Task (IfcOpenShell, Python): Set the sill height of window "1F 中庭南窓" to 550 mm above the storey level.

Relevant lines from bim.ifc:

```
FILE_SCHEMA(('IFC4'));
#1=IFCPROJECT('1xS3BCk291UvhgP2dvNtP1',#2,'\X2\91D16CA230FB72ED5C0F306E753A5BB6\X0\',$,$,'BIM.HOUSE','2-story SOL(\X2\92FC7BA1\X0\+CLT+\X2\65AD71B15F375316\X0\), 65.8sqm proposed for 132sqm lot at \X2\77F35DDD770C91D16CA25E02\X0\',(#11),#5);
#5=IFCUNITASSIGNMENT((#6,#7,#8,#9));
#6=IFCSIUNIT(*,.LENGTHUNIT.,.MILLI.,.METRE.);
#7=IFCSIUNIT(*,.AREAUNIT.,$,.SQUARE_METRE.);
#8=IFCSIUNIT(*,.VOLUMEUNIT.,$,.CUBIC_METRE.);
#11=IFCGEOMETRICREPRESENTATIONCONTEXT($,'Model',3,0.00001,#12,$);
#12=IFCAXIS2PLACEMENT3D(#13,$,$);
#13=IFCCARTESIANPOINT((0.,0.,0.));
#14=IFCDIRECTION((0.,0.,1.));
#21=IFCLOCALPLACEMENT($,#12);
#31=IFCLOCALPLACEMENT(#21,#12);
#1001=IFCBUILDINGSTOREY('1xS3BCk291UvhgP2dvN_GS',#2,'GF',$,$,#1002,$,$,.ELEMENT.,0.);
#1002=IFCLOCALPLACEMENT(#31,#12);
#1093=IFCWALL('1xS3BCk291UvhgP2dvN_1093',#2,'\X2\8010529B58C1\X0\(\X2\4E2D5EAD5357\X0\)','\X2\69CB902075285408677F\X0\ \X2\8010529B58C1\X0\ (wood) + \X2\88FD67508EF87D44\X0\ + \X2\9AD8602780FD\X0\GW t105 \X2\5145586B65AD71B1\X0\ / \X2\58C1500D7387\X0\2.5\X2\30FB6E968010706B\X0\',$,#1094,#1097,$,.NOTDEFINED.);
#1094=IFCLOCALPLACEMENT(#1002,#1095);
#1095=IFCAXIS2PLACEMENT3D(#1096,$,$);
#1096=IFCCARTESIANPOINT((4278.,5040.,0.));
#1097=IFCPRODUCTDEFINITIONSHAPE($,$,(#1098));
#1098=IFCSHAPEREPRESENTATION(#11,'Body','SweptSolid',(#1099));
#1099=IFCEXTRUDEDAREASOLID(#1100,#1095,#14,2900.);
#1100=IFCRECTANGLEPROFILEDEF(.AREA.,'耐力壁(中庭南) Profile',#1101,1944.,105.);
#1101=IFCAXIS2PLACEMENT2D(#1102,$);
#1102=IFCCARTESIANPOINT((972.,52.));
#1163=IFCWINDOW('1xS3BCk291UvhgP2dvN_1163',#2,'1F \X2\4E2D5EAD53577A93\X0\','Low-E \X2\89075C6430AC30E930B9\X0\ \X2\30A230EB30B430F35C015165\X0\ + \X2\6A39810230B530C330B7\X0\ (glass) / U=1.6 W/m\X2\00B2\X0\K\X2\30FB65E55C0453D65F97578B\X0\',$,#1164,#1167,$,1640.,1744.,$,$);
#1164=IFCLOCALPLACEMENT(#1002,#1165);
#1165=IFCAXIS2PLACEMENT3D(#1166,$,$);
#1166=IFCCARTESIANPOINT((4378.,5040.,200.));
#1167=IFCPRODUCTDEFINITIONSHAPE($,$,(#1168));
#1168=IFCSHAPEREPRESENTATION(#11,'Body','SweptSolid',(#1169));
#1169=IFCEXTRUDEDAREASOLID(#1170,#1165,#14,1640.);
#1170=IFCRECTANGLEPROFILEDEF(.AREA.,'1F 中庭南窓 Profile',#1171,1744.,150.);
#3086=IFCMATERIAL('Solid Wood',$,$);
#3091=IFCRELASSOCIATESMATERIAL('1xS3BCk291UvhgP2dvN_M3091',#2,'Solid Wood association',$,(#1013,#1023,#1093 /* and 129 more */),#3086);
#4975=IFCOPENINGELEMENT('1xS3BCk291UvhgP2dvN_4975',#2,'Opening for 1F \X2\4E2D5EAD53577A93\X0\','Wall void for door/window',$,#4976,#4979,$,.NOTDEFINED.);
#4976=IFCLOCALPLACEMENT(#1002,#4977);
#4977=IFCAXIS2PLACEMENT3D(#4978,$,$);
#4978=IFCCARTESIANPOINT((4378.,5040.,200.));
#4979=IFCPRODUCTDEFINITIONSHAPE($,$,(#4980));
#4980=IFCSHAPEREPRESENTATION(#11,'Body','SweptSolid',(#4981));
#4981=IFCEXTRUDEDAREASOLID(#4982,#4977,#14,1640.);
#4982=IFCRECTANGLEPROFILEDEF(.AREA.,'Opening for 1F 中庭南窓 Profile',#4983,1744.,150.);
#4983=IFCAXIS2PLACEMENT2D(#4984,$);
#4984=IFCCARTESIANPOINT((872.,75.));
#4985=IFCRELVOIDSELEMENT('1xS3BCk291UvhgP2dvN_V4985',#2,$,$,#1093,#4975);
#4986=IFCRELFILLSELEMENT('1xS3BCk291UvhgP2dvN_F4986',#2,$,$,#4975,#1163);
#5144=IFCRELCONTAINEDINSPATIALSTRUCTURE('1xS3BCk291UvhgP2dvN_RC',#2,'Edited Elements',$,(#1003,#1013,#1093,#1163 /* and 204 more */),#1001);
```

```python
import numpy as np
import ifcopenshell
import ifcopenshell.api.geometry
import ifcopenshell.geom
import ifcopenshell.util.element
import ifcopenshell.util.placement
import ifcopenshell.util.shape
import ifcopenshell.util.unit

model = ifcopenshell.open("bim.ifc")
unit_scale = ifcopenshell.util.unit.calculate_unit_scale(model)

window = model.by_guid("1xS3BCk291UvhgP2dvN_1163")
opening = window.FillsVoids[0].RelatingOpeningElement
storey = ifcopenshell.util.element.get_container(window, ifc_class="IfcBuildingStorey")
level = ifcopenshell.util.placement.get_local_placement(storey.ObjectPlacement)[2, 3]

# The opening's origin need not be at the sill, so measure its lowest point.
shape = ifcopenshell.geom.create_shape(ifcopenshell.geom.settings(), opening)
bottom = ifcopenshell.util.shape.get_shape_bottom_elevation(shape, shape.geometry) / unit_scale
dz = level + 550.0 - bottom

shift = np.array([0.0, 0.0, dz])
# The window is not placed relative to its opening, so move both.
for product in (opening, window):
    matrix = ifcopenshell.util.placement.get_local_placement(product.ObjectPlacement)
    matrix[:3, 3] += shift
    ifcopenshell.api.geometry.edit_object_placement(model, product=product, matrix=matrix, is_si=False)

print(f"moved by {dz * unit_scale:+.3f} m")

model.write("bim_v2.ifc")
```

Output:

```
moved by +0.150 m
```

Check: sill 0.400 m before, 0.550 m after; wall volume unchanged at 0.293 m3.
